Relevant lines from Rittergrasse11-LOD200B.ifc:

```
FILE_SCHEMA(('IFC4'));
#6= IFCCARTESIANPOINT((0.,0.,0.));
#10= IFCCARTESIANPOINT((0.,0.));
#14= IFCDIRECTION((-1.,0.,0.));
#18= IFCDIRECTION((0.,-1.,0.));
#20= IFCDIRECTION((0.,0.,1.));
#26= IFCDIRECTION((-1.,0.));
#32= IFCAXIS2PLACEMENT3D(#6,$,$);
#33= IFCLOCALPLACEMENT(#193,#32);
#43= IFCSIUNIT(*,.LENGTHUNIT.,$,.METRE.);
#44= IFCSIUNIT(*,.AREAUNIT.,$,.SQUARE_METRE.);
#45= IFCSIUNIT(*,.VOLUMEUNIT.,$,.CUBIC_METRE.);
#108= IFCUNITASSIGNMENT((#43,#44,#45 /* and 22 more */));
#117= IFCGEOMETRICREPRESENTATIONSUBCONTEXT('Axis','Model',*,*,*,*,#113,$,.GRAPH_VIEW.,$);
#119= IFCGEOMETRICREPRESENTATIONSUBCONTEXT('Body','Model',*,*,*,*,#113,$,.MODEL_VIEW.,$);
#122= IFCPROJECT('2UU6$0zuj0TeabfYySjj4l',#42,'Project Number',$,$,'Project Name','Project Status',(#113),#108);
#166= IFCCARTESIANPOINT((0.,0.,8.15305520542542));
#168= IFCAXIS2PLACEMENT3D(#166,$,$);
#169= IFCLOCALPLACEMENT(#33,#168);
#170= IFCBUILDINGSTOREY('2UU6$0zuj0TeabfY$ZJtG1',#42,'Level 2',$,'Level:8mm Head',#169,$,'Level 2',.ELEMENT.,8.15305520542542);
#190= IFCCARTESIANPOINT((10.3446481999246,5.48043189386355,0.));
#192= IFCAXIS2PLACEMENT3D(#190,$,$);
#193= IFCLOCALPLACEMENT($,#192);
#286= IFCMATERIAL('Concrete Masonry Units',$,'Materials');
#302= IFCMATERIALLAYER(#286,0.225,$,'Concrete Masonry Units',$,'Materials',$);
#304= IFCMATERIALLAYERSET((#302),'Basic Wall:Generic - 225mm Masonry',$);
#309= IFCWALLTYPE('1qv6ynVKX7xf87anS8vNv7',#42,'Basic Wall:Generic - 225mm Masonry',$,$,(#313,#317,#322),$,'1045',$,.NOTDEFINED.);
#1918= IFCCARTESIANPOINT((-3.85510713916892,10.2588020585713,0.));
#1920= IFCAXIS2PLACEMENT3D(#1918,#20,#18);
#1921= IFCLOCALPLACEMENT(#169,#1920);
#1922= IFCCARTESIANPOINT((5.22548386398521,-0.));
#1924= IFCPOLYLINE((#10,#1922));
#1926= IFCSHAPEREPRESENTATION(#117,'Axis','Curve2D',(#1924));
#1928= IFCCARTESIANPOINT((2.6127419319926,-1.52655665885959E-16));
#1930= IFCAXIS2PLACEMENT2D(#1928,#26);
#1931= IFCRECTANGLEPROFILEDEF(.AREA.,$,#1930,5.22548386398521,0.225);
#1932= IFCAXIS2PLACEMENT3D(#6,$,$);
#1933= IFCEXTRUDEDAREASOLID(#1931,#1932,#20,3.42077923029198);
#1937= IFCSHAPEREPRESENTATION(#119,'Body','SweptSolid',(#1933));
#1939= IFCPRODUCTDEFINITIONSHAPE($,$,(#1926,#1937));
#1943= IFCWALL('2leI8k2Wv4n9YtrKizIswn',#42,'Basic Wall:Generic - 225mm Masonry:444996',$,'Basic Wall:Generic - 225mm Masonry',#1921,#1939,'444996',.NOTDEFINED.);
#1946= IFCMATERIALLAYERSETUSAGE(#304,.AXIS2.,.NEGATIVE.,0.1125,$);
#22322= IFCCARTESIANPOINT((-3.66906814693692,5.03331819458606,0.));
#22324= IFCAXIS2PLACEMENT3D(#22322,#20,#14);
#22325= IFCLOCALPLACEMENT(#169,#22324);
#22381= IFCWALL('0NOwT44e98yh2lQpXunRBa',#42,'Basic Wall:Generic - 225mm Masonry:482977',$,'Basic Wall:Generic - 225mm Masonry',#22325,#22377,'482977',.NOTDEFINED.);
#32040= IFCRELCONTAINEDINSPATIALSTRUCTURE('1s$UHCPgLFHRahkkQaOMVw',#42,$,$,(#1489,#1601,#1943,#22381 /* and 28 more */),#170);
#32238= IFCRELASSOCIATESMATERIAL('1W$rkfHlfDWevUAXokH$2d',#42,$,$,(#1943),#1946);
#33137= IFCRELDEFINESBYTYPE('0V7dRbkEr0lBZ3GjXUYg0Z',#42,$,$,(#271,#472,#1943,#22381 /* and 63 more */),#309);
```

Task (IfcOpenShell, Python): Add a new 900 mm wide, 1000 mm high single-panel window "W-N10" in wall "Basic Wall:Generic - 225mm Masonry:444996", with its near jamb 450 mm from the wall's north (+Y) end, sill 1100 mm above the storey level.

```python
import numpy as np
import ifcopenshell
import ifcopenshell.api.feature
import ifcopenshell.api.geometry
import ifcopenshell.api.root
import ifcopenshell.api.spatial
import ifcopenshell.geom
import ifcopenshell.util.element
import ifcopenshell.util.placement
import ifcopenshell.util.representation
import ifcopenshell.util.shape
import ifcopenshell.util.unit

model = ifcopenshell.open("Rittergrasse11-LOD200B.ifc")
unit_scale = ifcopenshell.util.unit.calculate_unit_scale(model)
settings = ifcopenshell.geom.settings()


def volume(element):
    """Net volume in cubic metres, openings subtracted."""
    shape = ifcopenshell.geom.create_shape(settings, element)
    return ifcopenshell.util.shape.get_volume(shape.geometry)


wall = model.by_guid("2leI8k2Wv4n9YtrKizIswn")
storey = ifcopenshell.util.element.get_container(wall, ifc_class="IfcBuildingStorey")
context = ifcopenshell.util.representation.get_context(model, "Model", "Body", "MODEL_VIEW")
before = volume(wall)

width, height, from_end, sill = 0.9, 1, 0.45, 1.1  # metres

# The wall runs along its own X axis, and the end named is its -X end.
wall_shape = ifcopenshell.geom.create_shape(settings, wall)
x, y, z = ifcopenshell.util.shape.get_vertices(wall_shape.geometry).T
start = x.min() + from_end
face, thickness = float(y.min()), float(y.max() - y.min())
wall_matrix = ifcopenshell.util.placement.get_local_placement(wall.ObjectPlacement)
level = ifcopenshell.util.placement.get_local_placement(storey.ObjectPlacement)[2, 3]


def in_wall(x, y):
    """Placement at x, y metres in the wall's axes, at sill height."""
    matrix = wall_matrix.copy()
    matrix[:, 3] = wall_matrix @ np.array([x / unit_scale, y / unit_scale, 0.0, 1.0])
    matrix[2, 3] = level + sill / unit_scale
    return matrix


# Opening: a box that overshoots both wall faces by 50 mm.
opening = ifcopenshell.api.root.create_entity(model, ifc_class="IfcOpeningElement", predefined_type="OPENING")
box = ifcopenshell.api.geometry.add_wall_representation(
    model, context=context, length=width, height=height, thickness=thickness + 0.1
)
ifcopenshell.api.geometry.assign_representation(model, product=opening, representation=box)
ifcopenshell.api.geometry.edit_object_placement(model, product=opening, matrix=in_wall(start, face - 0.05), is_si=False)
ifcopenshell.api.feature.add_feature(model, feature=opening, element=wall)

window = ifcopenshell.api.root.create_entity(model, ifc_class="IfcWindow", name="W-N10", predefined_type="WINDOW")
window.OverallWidth, window.OverallHeight = width / unit_scale, height / unit_scale
window.PartitioningType = "SINGLE_PANEL"
body = ifcopenshell.api.geometry.add_window_representation(
    model,
    context=context,
    overall_width=window.OverallWidth,
    overall_height=window.OverallHeight,
    partition_type="SINGLE_PANEL",
)
ifcopenshell.api.geometry.assign_representation(model, product=window, representation=body)
ifcopenshell.api.spatial.assign_container(model, products=[window], relating_structure=storey)
ifcopenshell.api.feature.add_filling(model, opening=opening, element=window)

# Centre the window in the wall's thickness.
ifcopenshell.api.geometry.edit_object_placement(model, product=window, matrix=in_wall(start, face), is_si=False)
window_shape = ifcopenshell.geom.create_shape(settings, window)
depth = ifcopenshell.util.shape.get_vertices(window_shape.geometry)[:, 1]
offset = face + thickness / 2 - (depth.min() + depth.max()) / 2
ifcopenshell.api.geometry.edit_object_placement(model, product=window, matrix=in_wall(start, offset), is_si=False)

after = volume(wall)

print(f"wall volume {before:.3f} -> {after:.3f} m3")

model.write("Rittergrasse11-LOD200B_rev.ifc")
```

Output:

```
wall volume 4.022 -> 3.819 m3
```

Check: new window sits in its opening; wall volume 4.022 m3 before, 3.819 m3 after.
